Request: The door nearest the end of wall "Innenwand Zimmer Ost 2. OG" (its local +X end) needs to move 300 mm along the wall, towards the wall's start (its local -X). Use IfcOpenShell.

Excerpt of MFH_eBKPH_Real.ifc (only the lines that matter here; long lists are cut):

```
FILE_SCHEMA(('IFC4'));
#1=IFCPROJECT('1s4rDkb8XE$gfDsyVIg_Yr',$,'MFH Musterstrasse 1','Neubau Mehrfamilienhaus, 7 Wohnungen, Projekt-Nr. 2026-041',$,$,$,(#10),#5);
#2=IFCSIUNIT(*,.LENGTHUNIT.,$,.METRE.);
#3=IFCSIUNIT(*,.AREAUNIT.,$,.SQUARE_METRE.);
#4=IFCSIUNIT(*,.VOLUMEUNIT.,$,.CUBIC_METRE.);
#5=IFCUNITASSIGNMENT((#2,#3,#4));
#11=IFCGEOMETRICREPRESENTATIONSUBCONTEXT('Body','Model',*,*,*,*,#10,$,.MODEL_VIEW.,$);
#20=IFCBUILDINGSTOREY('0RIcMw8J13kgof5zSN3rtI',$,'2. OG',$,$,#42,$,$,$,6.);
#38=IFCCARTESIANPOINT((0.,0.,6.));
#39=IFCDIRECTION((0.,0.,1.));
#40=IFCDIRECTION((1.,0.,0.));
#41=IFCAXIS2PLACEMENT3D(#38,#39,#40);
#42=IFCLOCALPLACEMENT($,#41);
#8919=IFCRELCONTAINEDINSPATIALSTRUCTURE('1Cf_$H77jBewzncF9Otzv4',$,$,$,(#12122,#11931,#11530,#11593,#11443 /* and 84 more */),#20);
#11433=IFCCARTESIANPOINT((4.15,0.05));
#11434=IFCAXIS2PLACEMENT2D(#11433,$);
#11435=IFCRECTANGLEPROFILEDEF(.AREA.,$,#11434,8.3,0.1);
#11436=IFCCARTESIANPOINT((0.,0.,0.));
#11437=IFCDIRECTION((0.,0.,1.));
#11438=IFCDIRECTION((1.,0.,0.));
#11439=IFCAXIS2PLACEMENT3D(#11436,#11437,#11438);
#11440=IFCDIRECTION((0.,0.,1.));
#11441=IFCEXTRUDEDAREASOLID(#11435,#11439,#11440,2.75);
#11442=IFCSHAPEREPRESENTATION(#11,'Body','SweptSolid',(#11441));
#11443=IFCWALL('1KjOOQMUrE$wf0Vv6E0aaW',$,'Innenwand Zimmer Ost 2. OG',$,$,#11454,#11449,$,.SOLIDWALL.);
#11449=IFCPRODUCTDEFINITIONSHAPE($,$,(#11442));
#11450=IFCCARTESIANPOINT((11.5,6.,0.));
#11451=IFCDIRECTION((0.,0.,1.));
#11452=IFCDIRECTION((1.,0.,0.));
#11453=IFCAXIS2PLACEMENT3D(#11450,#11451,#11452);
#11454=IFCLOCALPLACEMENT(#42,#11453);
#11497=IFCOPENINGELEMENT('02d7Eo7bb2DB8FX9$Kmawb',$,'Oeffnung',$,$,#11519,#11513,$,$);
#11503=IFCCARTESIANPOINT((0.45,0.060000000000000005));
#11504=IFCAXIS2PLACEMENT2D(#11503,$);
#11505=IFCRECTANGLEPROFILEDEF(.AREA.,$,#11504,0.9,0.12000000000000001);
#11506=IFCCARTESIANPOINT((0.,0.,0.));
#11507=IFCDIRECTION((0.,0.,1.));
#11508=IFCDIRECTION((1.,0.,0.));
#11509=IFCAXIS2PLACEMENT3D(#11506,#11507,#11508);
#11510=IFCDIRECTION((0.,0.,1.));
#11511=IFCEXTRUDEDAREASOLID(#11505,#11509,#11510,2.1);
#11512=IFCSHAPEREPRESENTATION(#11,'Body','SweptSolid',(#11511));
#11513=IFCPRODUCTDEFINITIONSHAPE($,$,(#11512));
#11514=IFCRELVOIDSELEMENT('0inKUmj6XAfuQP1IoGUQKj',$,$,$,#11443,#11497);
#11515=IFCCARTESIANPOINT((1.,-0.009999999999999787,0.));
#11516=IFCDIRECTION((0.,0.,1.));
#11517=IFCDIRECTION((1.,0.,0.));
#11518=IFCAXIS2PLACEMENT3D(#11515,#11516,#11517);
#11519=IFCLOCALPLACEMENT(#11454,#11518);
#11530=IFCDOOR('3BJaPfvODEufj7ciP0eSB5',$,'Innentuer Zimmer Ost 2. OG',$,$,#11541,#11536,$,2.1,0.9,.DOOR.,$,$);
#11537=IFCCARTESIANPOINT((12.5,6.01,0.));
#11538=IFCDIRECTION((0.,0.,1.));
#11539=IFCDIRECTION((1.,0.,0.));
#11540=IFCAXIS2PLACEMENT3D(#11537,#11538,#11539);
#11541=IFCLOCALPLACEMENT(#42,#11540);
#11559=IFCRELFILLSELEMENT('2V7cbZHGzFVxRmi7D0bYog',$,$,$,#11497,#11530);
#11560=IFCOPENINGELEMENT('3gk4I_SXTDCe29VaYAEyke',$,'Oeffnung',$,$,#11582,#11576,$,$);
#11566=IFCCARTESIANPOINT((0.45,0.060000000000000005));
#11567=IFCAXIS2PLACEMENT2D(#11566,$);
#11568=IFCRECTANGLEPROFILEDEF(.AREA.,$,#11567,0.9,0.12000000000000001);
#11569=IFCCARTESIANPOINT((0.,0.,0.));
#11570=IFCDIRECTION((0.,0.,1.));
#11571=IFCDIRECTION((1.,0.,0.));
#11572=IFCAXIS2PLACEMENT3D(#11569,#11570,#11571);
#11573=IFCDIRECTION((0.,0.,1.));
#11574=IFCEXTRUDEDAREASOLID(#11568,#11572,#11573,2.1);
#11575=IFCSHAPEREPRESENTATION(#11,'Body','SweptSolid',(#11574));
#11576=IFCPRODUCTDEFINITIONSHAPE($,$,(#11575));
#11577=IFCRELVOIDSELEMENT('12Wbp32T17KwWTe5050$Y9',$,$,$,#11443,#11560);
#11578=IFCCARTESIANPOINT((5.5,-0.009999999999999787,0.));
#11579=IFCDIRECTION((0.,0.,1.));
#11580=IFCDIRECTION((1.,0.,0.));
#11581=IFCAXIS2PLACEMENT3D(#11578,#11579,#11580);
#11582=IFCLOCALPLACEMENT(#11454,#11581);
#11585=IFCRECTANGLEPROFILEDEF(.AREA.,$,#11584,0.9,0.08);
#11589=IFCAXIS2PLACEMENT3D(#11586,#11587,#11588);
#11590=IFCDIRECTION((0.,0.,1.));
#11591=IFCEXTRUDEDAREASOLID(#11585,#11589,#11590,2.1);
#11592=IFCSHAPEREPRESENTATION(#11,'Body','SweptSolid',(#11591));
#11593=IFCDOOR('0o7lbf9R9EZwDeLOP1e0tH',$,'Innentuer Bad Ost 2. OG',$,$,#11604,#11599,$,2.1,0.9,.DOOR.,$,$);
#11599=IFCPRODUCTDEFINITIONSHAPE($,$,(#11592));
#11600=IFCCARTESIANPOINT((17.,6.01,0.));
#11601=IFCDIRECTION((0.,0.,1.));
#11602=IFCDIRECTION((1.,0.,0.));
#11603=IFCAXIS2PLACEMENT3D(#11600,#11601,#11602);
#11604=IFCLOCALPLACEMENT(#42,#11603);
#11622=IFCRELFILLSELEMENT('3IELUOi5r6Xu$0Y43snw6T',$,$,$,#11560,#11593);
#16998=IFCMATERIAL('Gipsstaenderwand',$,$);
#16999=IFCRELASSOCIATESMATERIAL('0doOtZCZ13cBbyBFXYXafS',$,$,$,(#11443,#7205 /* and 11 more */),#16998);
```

```python
import ifcopenshell
import ifcopenshell.api.geometry
import ifcopenshell.util.placement
import ifcopenshell.util.unit

model = ifcopenshell.open("MFH_eBKPH_Real.ifc")
unit_scale = ifcopenshell.util.unit.calculate_unit_scale(model)

door = model.by_guid("0o7lbf9R9EZwDeLOP1e0tH")
opening = door.FillsVoids[0].RelatingOpeningElement
wall = opening.VoidsElements[0].RelatingBuildingElement

wall_matrix = ifcopenshell.util.placement.get_local_placement(wall.ObjectPlacement)
shift = wall_matrix[:3, 0] * -0.3 / unit_scale
before = ifcopenshell.util.placement.get_local_placement(door.ObjectPlacement)[:3, 3].copy()

# The door is not placed relative to its opening, so move both.
for product in (opening, door):
    matrix = ifcopenshell.util.placement.get_local_placement(product.ObjectPlacement)
    matrix[:3, 3] += shift
    ifcopenshell.api.geometry.edit_object_placement(model, product=product, matrix=matrix, is_si=False)

after = ifcopenshell.util.placement.get_local_placement(door.ObjectPlacement)[:3, 3]
print("door moved by", (after - before).round(3) + 0.0)

model.write("MFH_eBKPH_Real_rev.ifc")
```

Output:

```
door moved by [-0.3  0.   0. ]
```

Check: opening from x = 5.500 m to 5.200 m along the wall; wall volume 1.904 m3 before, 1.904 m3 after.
